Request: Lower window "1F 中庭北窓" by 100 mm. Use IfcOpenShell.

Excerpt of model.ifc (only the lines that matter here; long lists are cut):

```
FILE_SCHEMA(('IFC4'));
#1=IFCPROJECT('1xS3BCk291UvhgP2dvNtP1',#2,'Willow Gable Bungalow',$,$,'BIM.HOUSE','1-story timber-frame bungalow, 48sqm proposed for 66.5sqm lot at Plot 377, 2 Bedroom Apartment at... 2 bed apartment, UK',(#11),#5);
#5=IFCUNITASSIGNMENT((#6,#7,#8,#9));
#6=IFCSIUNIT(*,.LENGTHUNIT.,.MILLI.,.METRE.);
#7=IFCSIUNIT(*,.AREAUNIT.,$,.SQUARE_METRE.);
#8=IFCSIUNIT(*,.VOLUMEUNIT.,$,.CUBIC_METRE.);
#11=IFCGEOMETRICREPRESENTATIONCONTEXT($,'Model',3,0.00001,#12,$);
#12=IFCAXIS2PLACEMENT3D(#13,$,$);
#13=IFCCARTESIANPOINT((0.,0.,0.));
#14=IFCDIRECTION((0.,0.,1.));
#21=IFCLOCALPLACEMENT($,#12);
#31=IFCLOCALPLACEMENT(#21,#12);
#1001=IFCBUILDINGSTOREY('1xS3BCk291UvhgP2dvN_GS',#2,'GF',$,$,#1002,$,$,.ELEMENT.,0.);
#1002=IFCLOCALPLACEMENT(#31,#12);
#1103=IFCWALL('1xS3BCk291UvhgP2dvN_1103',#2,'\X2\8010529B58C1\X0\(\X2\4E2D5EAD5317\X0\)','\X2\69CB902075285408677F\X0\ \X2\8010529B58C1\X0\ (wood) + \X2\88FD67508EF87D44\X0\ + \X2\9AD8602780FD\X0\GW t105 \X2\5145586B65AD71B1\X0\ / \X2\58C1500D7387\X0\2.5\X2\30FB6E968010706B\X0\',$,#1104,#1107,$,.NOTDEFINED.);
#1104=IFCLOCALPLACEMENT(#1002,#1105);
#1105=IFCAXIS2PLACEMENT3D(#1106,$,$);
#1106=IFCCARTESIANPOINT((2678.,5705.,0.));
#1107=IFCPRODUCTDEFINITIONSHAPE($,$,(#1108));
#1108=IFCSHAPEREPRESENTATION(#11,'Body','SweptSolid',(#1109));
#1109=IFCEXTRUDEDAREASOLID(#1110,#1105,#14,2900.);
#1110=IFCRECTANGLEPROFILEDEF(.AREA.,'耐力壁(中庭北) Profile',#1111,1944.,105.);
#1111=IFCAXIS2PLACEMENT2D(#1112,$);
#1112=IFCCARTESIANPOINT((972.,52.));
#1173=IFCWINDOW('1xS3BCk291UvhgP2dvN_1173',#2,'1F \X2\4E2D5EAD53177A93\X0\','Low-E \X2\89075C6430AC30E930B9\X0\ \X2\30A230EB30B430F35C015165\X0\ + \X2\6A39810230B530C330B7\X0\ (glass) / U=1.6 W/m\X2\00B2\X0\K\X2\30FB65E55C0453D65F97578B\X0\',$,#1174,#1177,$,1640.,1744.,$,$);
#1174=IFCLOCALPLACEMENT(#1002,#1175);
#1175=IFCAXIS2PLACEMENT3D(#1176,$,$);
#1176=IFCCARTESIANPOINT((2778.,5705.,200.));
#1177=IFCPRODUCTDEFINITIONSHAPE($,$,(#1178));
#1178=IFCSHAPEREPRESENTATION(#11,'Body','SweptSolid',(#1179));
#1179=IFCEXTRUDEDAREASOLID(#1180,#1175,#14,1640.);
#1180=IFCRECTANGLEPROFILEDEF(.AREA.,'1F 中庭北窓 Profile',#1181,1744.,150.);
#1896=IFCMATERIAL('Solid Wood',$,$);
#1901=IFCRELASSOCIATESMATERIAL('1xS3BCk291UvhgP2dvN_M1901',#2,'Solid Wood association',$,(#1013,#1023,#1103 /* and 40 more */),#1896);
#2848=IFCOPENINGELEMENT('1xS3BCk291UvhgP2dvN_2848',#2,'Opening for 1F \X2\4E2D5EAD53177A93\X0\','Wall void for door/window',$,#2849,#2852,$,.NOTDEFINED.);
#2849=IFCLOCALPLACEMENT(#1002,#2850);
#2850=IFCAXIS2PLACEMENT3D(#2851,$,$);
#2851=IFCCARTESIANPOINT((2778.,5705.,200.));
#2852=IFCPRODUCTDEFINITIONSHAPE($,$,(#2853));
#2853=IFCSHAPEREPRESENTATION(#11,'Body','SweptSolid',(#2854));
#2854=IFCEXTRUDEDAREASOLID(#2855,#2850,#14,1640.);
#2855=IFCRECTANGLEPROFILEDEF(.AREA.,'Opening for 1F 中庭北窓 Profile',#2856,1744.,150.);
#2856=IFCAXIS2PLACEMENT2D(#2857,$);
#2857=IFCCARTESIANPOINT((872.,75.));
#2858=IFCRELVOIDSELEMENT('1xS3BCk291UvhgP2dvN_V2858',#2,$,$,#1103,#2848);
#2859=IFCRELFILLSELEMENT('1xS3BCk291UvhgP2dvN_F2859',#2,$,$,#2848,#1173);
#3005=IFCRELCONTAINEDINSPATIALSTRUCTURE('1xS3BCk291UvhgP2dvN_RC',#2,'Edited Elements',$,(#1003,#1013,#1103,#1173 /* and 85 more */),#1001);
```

```python
import numpy as np
import ifcopenshell
import ifcopenshell.api.geometry
import ifcopenshell.util.placement
import ifcopenshell.util.unit

model = ifcopenshell.open("model.ifc")
unit_scale = ifcopenshell.util.unit.calculate_unit_scale(model)

window = model.by_guid("1xS3BCk291UvhgP2dvN_1173")
opening = window.FillsVoids[0].RelatingOpeningElement
dz = -0.1 / unit_scale

shift = np.array([0.0, 0.0, dz])
# The window is not placed relative to its opening, so move both.
for product in (opening, window):
    matrix = ifcopenshell.util.placement.get_local_placement(product.ObjectPlacement)
    matrix[:3, 3] += shift
    ifcopenshell.api.geometry.edit_object_placement(model, product=product, matrix=matrix, is_si=False)

print(f"moved by {dz * unit_scale:+.3f} m")

model.write("model_edited.ifc")
```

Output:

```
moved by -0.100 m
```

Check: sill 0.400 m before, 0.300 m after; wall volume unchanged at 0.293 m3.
